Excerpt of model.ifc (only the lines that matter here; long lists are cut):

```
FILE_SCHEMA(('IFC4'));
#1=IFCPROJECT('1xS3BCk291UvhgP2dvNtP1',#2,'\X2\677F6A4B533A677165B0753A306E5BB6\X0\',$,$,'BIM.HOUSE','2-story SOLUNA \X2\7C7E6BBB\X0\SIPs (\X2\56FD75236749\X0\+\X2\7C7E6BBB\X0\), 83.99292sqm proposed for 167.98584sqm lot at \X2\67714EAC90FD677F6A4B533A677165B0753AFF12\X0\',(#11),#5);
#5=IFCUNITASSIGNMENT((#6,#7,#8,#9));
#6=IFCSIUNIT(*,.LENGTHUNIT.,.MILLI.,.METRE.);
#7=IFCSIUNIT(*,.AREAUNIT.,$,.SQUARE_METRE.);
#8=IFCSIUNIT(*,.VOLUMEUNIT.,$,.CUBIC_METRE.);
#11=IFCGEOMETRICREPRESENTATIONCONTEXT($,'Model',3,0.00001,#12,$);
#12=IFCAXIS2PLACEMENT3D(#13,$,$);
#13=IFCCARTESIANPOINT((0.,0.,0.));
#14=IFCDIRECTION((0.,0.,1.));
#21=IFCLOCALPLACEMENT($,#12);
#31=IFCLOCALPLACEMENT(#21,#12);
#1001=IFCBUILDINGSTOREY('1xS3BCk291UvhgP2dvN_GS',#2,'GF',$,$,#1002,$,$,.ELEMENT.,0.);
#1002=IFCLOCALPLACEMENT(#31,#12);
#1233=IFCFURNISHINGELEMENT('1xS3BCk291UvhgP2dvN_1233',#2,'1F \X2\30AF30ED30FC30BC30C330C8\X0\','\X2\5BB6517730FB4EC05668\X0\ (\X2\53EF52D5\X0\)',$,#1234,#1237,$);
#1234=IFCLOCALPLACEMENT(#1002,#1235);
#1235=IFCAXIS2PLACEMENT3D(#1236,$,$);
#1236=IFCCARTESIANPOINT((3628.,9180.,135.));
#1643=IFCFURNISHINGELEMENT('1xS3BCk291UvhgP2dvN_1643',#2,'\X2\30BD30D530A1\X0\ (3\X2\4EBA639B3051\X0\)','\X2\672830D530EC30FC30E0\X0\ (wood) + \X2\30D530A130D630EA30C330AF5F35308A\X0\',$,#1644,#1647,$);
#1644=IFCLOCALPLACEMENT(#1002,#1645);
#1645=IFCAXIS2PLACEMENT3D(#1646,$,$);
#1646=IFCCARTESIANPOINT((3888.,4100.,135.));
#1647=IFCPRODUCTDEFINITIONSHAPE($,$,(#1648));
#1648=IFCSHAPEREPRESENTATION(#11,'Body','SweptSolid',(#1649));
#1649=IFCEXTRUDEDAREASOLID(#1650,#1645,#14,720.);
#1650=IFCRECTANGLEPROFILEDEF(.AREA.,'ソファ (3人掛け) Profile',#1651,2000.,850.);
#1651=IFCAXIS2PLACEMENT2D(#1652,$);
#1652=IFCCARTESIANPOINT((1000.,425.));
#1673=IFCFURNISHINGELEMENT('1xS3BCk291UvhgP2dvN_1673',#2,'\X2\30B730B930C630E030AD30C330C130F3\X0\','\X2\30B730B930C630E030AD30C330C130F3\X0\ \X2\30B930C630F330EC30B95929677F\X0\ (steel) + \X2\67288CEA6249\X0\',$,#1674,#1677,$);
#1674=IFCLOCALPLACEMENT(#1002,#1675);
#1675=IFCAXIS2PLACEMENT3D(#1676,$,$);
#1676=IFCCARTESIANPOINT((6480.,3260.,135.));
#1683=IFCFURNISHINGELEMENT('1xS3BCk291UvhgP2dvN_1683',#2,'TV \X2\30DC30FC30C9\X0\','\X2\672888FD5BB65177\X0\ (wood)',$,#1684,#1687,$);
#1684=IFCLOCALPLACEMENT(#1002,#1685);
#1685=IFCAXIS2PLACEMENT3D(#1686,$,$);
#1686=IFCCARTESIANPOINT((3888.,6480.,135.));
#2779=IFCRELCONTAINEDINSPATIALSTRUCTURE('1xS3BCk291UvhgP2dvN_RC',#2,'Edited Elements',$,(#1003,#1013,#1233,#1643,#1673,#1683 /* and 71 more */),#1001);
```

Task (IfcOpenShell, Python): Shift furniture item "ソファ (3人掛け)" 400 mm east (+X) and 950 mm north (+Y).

```python
import ifcopenshell
import ifcopenshell.api.geometry
import ifcopenshell.util.placement
import ifcopenshell.util.unit

model = ifcopenshell.open("model.ifc")
unit_scale = ifcopenshell.util.unit.calculate_unit_scale(model)

item = model.by_id(1643)
matrix = ifcopenshell.util.placement.get_local_placement(item.ObjectPlacement)
matrix[0, 3] += 0.4 / unit_scale
matrix[1, 3] += 0.95 / unit_scale
ifcopenshell.api.geometry.edit_object_placement(model, product=item, matrix=matrix, is_si=False)

print(ifcopenshell.util.placement.get_local_placement(item.ObjectPlacement).round(3) + 0.0)

model.write("model_updated.ifc")
```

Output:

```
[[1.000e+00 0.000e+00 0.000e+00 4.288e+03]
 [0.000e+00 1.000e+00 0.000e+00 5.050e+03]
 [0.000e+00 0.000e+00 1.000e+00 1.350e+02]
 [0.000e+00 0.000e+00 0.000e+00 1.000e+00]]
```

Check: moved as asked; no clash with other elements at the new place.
